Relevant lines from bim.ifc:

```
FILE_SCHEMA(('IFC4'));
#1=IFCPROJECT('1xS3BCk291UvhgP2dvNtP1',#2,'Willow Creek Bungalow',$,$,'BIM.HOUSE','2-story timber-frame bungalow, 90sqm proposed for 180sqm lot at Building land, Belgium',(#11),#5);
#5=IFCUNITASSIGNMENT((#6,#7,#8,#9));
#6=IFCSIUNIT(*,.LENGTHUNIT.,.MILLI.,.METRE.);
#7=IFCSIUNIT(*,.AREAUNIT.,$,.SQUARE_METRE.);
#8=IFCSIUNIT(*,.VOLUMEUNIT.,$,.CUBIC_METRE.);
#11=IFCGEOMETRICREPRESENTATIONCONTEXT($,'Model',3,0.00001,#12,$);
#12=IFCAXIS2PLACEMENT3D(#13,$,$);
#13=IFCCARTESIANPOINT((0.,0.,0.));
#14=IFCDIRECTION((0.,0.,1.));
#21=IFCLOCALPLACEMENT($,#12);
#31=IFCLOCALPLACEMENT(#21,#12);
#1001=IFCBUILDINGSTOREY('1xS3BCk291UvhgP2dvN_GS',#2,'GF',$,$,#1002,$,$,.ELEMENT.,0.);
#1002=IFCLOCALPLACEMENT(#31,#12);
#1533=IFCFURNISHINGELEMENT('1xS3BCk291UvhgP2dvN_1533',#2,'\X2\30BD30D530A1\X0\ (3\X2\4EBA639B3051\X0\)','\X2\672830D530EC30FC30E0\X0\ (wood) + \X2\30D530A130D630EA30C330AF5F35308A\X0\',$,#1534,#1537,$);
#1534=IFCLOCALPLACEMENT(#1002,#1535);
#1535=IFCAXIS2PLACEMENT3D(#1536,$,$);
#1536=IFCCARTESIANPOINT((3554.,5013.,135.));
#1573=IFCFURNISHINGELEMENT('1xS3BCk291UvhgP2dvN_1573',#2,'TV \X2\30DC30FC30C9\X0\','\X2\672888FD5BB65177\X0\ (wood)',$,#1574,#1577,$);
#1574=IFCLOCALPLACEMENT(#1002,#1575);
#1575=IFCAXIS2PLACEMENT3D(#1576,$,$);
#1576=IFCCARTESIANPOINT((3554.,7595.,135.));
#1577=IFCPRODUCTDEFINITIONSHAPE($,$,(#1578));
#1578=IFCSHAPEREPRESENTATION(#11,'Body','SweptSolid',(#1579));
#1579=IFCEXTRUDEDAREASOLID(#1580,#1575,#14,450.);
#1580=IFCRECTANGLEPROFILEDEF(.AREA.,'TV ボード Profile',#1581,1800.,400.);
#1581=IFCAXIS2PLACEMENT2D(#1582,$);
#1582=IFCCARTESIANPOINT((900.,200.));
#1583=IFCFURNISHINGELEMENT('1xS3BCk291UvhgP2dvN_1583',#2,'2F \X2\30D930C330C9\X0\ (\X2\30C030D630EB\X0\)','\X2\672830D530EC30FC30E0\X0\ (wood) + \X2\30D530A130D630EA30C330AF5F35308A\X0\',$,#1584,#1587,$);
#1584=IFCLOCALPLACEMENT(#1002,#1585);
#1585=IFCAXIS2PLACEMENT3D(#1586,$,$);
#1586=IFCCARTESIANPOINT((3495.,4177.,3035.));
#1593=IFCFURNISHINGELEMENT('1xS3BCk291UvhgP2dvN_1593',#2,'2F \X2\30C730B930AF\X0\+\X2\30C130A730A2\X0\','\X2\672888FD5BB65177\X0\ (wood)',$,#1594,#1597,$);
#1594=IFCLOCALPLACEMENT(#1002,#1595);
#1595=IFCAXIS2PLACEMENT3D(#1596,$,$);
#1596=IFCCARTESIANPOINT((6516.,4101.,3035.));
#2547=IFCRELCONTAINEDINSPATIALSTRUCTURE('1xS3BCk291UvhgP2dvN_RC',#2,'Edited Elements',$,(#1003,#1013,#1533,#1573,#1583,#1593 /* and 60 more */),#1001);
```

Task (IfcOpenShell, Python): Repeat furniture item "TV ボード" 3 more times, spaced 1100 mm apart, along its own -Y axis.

```python
import ifcopenshell
import ifcopenshell.api.geometry
import ifcopenshell.api.root
import ifcopenshell.util.element
import ifcopenshell.util.placement

model = ifcopenshell.open("bim.ifc")


def reuse_history(source, copy):
    """copy_class also copies each property set's owner history, people and application; keep the originals."""
    for rel in copy.IsDefinedBy:
        if rel.is_a("IfcRelDefinesByProperties") and (history := rel.RelatingPropertyDefinition.OwnerHistory):
            rel.RelatingPropertyDefinition.OwnerHistory = source.OwnerHistory
            ifcopenshell.util.element.remove_deep2(model, history)


source = model.by_id(1573)
base = ifcopenshell.util.placement.get_local_placement(source.ObjectPlacement)
step = -base[:3, 1] * 1100.0

for i in range(1, 4):
    copy = ifcopenshell.api.root.copy_class(model, product=source)
    copy.Representation = ifcopenshell.util.element.copy_deep(
        model, source.Representation, exclude=["IfcGeometricRepresentationContext", "IfcRepresentationMap"]
    )
    reuse_history(source, copy)
    matrix = base.copy()
    matrix[:3, 3] += i * step
    print("added at", matrix[:3, 3].round(3) + 0.0)
    ifcopenshell.api.geometry.edit_object_placement(model, product=copy, matrix=matrix, is_si=False)

model.write("bim_edited.ifc")
```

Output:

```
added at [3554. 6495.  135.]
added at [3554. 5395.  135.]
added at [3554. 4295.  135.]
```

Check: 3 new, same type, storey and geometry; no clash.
